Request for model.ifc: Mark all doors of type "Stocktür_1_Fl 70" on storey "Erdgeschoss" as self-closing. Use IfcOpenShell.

First a look at what the model holds.

```python
import ifcopenshell
import ifcopenshell.util.element

model = ifcopenshell.open("model.ifc")
print(model.schema)
storey = next(s for s in model.by_type("IfcBuildingStorey") if s.Name == "Erdgeschoss")
doors = [e for e in ifcopenshell.util.element.get_decomposition(storey) if e.is_a("IfcDoor")]
seen = {}
for e in doors:
    element_type = ifcopenshell.util.element.get_type(e)
    key = (element_type.Name if element_type != e and element_type else None, ifcopenshell.util.element.get_pset(e, "Pset_DoorCommon", "SelfClosing"))
    seen[key] = seen.get(key, 0) + 1
for (name, value), count in sorted(seen.items(), key=str):
    print(count, "x", name, "|", value)
```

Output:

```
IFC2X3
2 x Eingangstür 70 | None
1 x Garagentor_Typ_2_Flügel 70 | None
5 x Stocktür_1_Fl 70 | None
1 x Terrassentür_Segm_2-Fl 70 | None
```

```python
import ifcopenshell
import ifcopenshell.api.pset
import ifcopenshell.util.element

model = ifcopenshell.open("model.ifc")

storey = next(s for s in model.by_type("IfcBuildingStorey") if s.Name == "Erdgeschoss")
doors = [e for e in ifcopenshell.util.element.get_decomposition(storey) if e.is_a("IfcDoor")]

count = 0
for e in doors:
    element_type = ifcopenshell.util.element.get_type(e)
    if element_type in (None, e) or element_type.Name != "Stocktür_1_Fl 70":
        continue
    # add_pset returns the element's existing set when there is one.
    pset = ifcopenshell.api.pset.add_pset(model, product=e, name="Pset_DoorCommon")
    ifcopenshell.api.pset.edit_pset(model, pset=pset, properties={"SelfClosing": True})
    count += 1

print(count, "doors updated")

model.write("model_rev.ifc")
```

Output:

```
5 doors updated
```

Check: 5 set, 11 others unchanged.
